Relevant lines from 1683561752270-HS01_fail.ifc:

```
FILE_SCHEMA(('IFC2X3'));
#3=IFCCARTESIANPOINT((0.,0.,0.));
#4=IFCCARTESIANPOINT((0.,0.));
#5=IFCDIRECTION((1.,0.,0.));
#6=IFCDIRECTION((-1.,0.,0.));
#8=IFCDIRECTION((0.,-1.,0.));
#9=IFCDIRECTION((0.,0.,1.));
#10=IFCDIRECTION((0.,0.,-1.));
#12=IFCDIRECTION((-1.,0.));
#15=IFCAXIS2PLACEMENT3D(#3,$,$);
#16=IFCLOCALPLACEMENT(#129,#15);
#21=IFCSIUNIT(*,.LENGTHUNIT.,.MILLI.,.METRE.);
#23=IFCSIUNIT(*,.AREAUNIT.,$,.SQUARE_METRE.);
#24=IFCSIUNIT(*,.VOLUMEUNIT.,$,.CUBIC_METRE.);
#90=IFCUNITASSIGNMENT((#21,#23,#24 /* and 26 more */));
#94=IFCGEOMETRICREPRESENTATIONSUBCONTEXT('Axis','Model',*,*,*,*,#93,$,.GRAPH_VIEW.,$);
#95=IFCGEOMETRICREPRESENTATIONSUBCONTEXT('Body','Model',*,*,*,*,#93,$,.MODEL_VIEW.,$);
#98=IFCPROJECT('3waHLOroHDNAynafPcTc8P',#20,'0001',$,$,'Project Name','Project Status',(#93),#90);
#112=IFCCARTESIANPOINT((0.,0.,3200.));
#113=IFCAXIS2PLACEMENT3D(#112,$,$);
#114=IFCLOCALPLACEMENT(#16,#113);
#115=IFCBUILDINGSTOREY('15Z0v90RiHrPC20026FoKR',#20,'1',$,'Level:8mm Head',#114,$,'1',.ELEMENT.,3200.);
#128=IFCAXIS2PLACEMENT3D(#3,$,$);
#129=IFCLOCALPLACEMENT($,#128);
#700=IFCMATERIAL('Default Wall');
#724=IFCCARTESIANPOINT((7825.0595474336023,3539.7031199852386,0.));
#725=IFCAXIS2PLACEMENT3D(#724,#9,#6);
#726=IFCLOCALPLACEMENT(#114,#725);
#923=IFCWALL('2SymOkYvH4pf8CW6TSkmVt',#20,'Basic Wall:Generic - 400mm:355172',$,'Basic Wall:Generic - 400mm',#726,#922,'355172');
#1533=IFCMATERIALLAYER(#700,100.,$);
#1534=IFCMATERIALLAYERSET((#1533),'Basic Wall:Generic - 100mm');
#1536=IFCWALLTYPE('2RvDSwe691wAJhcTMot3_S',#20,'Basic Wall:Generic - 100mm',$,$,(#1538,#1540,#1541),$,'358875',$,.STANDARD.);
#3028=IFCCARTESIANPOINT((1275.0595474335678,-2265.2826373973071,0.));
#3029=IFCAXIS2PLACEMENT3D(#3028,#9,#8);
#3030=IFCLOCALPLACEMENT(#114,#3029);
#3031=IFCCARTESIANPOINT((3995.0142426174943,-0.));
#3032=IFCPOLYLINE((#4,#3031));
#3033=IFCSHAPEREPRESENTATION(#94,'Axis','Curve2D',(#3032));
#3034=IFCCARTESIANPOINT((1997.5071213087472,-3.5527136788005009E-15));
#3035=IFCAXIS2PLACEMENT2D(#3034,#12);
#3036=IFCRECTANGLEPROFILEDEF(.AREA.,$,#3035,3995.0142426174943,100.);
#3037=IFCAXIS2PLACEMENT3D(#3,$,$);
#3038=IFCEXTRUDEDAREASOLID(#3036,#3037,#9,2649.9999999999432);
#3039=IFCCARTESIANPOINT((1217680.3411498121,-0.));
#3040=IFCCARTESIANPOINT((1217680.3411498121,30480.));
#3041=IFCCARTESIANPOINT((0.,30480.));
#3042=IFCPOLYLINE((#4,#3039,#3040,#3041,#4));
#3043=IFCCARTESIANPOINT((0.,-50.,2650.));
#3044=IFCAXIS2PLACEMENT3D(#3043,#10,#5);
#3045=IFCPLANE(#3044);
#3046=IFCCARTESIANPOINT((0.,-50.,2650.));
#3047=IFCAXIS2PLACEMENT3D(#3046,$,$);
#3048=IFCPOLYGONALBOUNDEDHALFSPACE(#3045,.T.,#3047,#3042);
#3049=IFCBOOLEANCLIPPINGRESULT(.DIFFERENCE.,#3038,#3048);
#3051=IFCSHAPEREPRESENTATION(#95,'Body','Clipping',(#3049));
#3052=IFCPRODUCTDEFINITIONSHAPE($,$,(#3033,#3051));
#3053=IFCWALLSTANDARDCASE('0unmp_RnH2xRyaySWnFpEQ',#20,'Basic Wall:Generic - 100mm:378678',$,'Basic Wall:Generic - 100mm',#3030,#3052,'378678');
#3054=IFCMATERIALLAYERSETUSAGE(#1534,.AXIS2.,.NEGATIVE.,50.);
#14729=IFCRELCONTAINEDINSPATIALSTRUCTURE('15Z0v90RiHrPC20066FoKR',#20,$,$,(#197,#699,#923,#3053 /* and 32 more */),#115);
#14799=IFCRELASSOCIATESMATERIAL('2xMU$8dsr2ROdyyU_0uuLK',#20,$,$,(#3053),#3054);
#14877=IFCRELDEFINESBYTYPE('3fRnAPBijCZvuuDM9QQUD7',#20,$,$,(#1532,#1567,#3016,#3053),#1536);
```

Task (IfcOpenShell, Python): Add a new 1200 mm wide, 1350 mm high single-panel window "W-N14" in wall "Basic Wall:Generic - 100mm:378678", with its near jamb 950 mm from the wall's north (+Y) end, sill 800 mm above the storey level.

```python
import numpy as np
import ifcopenshell
import ifcopenshell.api.feature
import ifcopenshell.api.geometry
import ifcopenshell.api.root
import ifcopenshell.api.spatial
import ifcopenshell.api.type
import ifcopenshell.geom
import ifcopenshell.util.element
import ifcopenshell.util.placement
import ifcopenshell.util.representation
import ifcopenshell.util.shape
import ifcopenshell.util.unit

model = ifcopenshell.open("1683561752270-HS01_fail.ifc")
unit_scale = ifcopenshell.util.unit.calculate_unit_scale(model)
settings = ifcopenshell.geom.settings()


def volume(element):
    """Net volume in cubic metres, openings subtracted."""
    shape = ifcopenshell.geom.create_shape(settings, element)
    return ifcopenshell.util.shape.get_volume(shape.geometry)


wall = model.by_guid("0unmp_RnH2xRyaySWnFpEQ")
storey = ifcopenshell.util.element.get_container(wall, ifc_class="IfcBuildingStorey")
context = ifcopenshell.util.representation.get_context(model, "Model", "Body", "MODEL_VIEW")
before = volume(wall)

width, height, from_end, sill = 1.2, 1.35, 0.95, 0.8  # metres

# The wall runs along its own X axis, and the end named is its -X end.
wall_shape = ifcopenshell.geom.create_shape(settings, wall)
x, y, z = ifcopenshell.util.shape.get_vertices(wall_shape.geometry).T
start = x.min() + from_end
face, thickness = float(y.min()), float(y.max() - y.min())
wall_matrix = ifcopenshell.util.placement.get_local_placement(wall.ObjectPlacement)
level = ifcopenshell.util.placement.get_local_placement(storey.ObjectPlacement)[2, 3]


def in_wall(x, y):
    """Placement at x, y metres in the wall's axes, at sill height."""
    matrix = wall_matrix.copy()
    matrix[:, 3] = wall_matrix @ np.array([x / unit_scale, y / unit_scale, 0.0, 1.0])
    matrix[2, 3] = level + sill / unit_scale
    return matrix


# Opening: a box that overshoots both wall faces by 50 mm.
opening = ifcopenshell.api.root.create_entity(model, ifc_class="IfcOpeningElement")
box = ifcopenshell.api.geometry.add_wall_representation(
    model, context=context, length=width, height=height, thickness=thickness + 0.1
)
ifcopenshell.api.geometry.assign_representation(model, product=opening, representation=box)
ifcopenshell.api.geometry.edit_object_placement(model, product=opening, matrix=in_wall(start, face - 0.05), is_si=False)
ifcopenshell.api.feature.add_feature(model, feature=opening, element=wall)

window = ifcopenshell.api.root.create_entity(model, ifc_class="IfcWindow", name="W-N14")
window.OverallWidth, window.OverallHeight = width / unit_scale, height / unit_scale
body = ifcopenshell.api.geometry.add_window_representation(
    model,
    context=context,
    overall_width=window.OverallWidth,
    overall_height=window.OverallHeight,
    partition_type="SINGLE_PANEL",
)
ifcopenshell.api.geometry.assign_representation(model, product=window, representation=body)
ifcopenshell.api.spatial.assign_container(model, products=[window], relating_structure=storey)
fills = ifcopenshell.api.feature.add_filling(model, opening=opening, element=window)
fills.OwnerHistory = window.OwnerHistory  # required in IFC2X3

# IFC2X3 keeps the operation on the window style.
style = ifcopenshell.api.root.create_entity(model, ifc_class="IfcWindowStyle", name="W-N14")
style.OperationType, style.ConstructionType = "SINGLE_PANEL", "NOTDEFINED"
style.ParameterTakesPrecedence = style.Sizeable = False
ifcopenshell.api.type.assign_type(model, related_objects=[window], relating_type=style)

# Centre the window in the wall's thickness.
ifcopenshell.api.geometry.edit_object_placement(model, product=window, matrix=in_wall(start, face), is_si=False)
window_shape = ifcopenshell.geom.create_shape(settings, window)
depth = ifcopenshell.util.shape.get_vertices(window_shape.geometry)[:, 1]
offset = face + thickness / 2 - (depth.min() + depth.max()) / 2
ifcopenshell.api.geometry.edit_object_placement(model, product=window, matrix=in_wall(start, offset), is_si=False)

after = volume(wall)

print(f"wall volume {before:.3f} -> {after:.3f} m3")

model.write("1683561752270-HS01_fail_edited.ifc")
```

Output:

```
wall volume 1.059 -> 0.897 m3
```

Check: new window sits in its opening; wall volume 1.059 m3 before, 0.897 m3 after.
